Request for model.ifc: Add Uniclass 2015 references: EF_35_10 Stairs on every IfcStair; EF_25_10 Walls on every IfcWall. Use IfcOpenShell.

First a look at what the model holds.

```python
import ifcopenshell

model = ifcopenshell.open("model.ifc")
print(model.schema)
print("classifications:", [c.Name for c in model.by_type("IfcClassification")])
for ifc_class in ("IfcDoor", "IfcRoof", "IfcStair", "IfcWall", "IfcWindow"):
    print(ifc_class, len(model.by_type(ifc_class)))
```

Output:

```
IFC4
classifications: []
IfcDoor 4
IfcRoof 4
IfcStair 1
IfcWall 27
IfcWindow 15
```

```python
import ifcopenshell
import ifcopenshell.api.classification

model = ifcopenshell.open("model.ifc")

system = ifcopenshell.api.classification.add_classification(model, classification="Uniclass 2015")

codes = {
    "IfcStair": ("EF_35_10", "Stairs"),
    "IfcWall": ("EF_25_10", "Walls"),
}
for ifc_class, (code, name) in codes.items():
    products = model.by_type(ifc_class)
    ifcopenshell.api.classification.add_reference(
        model, products=products, classification=system, identification=code, name=name
    )
    print(code, len(products))

model.write("model_rev.ifc")
```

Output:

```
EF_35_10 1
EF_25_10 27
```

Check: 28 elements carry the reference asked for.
